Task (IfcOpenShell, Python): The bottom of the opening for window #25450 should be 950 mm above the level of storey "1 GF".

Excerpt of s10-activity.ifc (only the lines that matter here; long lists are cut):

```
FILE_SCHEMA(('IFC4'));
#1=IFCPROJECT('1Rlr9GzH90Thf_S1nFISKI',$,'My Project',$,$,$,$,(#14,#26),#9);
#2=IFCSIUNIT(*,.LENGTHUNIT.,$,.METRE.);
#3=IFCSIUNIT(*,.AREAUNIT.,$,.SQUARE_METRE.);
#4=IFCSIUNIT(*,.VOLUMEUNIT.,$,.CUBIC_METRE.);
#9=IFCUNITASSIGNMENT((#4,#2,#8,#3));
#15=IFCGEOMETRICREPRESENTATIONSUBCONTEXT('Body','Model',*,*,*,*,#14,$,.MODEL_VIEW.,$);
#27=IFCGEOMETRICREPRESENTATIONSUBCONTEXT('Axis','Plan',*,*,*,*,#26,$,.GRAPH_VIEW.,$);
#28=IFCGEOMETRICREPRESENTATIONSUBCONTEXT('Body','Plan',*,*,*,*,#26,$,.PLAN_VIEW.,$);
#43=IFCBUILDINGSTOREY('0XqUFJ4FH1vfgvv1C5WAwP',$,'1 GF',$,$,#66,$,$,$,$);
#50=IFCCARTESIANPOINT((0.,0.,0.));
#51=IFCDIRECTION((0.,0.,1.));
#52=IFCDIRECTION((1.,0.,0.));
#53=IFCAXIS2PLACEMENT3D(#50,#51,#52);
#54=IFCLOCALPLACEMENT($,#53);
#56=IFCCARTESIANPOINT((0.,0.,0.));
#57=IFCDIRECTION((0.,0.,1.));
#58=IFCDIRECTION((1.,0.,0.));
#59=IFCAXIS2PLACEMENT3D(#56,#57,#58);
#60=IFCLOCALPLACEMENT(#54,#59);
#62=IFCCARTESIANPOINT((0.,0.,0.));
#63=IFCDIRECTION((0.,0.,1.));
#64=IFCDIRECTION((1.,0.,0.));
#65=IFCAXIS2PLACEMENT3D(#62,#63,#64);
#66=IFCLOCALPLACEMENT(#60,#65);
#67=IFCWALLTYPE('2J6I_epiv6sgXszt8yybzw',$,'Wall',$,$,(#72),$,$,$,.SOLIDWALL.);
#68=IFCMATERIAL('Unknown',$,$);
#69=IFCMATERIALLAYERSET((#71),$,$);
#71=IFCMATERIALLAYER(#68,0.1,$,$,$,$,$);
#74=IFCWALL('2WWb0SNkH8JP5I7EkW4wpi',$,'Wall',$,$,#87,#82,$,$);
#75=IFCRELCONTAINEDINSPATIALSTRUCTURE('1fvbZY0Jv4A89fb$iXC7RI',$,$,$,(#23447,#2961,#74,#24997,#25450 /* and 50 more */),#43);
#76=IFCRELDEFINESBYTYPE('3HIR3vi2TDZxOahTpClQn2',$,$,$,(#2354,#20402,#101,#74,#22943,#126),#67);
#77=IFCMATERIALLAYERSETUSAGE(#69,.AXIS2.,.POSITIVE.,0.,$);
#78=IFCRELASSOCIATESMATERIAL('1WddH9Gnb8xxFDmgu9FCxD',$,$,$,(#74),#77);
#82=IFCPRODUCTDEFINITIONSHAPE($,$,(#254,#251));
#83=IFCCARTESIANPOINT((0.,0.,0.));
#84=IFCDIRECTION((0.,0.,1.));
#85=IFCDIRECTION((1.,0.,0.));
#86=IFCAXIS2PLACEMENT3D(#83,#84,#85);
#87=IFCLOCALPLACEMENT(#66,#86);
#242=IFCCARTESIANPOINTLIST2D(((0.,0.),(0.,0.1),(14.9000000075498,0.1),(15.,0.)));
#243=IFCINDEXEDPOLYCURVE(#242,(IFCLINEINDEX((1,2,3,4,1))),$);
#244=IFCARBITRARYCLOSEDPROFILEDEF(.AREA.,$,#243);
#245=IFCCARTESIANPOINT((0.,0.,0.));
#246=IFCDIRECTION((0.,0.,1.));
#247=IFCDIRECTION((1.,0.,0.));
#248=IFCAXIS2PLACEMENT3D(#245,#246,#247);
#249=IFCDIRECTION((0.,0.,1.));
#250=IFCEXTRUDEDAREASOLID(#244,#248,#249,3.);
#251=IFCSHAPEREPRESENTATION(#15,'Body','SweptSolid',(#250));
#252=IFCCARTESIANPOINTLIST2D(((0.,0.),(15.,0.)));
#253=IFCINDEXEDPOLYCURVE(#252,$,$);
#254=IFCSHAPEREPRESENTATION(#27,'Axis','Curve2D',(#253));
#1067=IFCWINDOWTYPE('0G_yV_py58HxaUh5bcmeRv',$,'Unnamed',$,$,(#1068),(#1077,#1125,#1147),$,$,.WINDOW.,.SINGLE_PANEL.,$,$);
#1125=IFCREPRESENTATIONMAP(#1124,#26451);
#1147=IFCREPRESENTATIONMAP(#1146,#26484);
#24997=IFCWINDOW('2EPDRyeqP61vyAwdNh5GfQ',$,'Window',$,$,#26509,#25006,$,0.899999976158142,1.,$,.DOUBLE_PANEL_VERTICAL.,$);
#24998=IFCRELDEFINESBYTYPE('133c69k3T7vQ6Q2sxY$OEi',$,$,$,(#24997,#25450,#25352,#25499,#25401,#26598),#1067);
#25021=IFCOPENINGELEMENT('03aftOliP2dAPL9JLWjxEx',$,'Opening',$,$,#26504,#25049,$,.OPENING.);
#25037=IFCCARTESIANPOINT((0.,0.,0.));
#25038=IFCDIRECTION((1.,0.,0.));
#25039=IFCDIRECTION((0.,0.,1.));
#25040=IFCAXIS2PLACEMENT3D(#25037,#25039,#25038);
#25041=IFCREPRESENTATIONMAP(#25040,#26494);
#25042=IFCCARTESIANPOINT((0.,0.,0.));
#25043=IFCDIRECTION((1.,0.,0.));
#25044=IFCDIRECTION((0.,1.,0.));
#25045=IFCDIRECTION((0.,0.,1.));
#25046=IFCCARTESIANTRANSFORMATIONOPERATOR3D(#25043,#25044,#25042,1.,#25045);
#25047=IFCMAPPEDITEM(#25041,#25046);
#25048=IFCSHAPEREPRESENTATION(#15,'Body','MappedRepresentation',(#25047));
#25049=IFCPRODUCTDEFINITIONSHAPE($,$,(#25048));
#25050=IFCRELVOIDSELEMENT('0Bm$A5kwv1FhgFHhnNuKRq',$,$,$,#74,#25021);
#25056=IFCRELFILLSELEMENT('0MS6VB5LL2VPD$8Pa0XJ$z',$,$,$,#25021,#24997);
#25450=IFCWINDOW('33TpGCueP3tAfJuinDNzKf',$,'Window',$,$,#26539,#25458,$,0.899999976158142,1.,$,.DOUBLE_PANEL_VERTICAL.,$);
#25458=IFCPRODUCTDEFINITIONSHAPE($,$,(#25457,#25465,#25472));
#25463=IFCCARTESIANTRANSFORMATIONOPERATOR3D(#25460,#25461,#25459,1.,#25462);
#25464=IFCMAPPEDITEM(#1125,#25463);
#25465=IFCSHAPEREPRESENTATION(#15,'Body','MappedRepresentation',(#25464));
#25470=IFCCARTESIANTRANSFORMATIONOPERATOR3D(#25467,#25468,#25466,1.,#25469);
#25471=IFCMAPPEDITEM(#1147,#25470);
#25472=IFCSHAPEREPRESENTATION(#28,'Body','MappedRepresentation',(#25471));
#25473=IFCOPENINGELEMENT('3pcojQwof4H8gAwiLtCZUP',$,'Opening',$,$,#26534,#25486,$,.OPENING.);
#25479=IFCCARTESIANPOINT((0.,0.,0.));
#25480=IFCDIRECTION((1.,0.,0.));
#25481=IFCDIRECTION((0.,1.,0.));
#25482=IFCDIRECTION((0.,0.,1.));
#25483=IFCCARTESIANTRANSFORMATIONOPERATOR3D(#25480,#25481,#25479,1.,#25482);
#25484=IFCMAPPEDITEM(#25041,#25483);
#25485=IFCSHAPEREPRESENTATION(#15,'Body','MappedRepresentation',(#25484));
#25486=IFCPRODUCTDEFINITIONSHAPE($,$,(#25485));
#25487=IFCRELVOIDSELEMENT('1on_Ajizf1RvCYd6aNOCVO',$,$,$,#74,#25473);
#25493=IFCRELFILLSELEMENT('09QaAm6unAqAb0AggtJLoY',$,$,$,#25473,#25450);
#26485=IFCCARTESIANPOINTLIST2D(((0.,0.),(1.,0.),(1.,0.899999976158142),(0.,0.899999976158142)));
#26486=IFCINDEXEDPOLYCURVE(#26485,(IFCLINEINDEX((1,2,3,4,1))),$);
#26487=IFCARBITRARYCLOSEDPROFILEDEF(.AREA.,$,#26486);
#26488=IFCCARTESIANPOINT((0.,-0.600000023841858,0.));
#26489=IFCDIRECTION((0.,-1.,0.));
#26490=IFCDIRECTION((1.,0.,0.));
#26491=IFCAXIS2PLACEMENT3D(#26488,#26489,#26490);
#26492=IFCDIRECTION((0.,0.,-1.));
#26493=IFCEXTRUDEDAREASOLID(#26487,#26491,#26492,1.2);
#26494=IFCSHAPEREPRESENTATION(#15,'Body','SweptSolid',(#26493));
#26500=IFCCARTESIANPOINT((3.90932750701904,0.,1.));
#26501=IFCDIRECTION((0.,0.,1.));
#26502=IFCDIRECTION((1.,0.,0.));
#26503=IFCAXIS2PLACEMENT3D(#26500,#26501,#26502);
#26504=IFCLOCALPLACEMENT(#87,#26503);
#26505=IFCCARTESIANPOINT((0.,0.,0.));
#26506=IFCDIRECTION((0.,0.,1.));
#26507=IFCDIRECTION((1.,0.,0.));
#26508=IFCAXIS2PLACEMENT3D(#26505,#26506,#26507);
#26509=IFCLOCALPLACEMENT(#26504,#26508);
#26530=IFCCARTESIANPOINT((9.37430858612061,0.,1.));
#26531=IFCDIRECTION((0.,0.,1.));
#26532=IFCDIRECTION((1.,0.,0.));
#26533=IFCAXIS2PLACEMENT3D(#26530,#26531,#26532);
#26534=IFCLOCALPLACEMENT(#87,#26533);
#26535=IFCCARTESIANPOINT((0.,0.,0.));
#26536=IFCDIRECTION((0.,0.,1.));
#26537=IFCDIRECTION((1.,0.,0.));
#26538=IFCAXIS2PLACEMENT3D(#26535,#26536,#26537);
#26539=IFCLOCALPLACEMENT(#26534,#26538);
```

```python
import numpy as np
import ifcopenshell
import ifcopenshell.api.geometry
import ifcopenshell.geom
import ifcopenshell.util.element
import ifcopenshell.util.placement
import ifcopenshell.util.shape
import ifcopenshell.util.unit

model = ifcopenshell.open("s10-activity.ifc")
unit_scale = ifcopenshell.util.unit.calculate_unit_scale(model)

window = model.by_id(25450)
opening = window.FillsVoids[0].RelatingOpeningElement
storey = ifcopenshell.util.element.get_container(window, ifc_class="IfcBuildingStorey")
level = ifcopenshell.util.placement.get_local_placement(storey.ObjectPlacement)[2, 3]

# The opening's origin need not be at the sill, so measure its lowest point.
shape = ifcopenshell.geom.create_shape(ifcopenshell.geom.settings(), opening)
bottom = ifcopenshell.util.shape.get_shape_bottom_elevation(shape, shape.geometry) / unit_scale
dz = level + 0.95 - bottom

shift = np.array([0.0, 0.0, dz])
# The window is placed relative to its opening, so it follows when the opening moves.
matrix = ifcopenshell.util.placement.get_local_placement(opening.ObjectPlacement)
matrix[:3, 3] += shift
ifcopenshell.api.geometry.edit_object_placement(
    model, product=opening, matrix=matrix, is_si=False, should_transform_children=True
)

print(f"moved by {dz * unit_scale:+.3f} m")

model.write("s10-activity-out.ifc")
```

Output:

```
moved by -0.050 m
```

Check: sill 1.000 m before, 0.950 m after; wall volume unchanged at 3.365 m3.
